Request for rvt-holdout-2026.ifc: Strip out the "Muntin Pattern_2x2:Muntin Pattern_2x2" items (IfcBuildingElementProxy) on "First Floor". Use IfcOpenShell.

First a look at what the model holds.

```python
import ifcopenshell
import ifcopenshell.util.element

model = ifcopenshell.open("rvt-holdout-2026.ifc")
print(model.schema)
storey = next(s for s in model.by_type("IfcBuildingStorey") if s.Name == "First Floor")
proxies = [e for e in ifcopenshell.util.element.get_decomposition(storey) if e.is_a("IfcBuildingElementProxy")]
seen = {}
for e in proxies:
    element_type = ifcopenshell.util.element.get_type(e)
    name = element_type.Name if element_type not in (None, e) else None
    seen[name] = seen.get(name, 0) + 1
for name, count in sorted(seen.items(), key=str):
    print(count, "x", name)
```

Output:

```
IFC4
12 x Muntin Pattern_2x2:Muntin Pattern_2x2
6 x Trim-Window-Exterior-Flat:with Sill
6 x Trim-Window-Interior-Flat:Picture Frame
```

```python
import ifcopenshell
import ifcopenshell.api.root
import ifcopenshell.util.element

model = ifcopenshell.open("rvt-holdout-2026.ifc")

storey = next(s for s in model.by_type("IfcBuildingStorey") if s.Name == "First Floor")
proxies = [e for e in ifcopenshell.util.element.get_decomposition(storey) if e.is_a("IfcBuildingElementProxy")]
targets = [e for e in proxies if (t := ifcopenshell.util.element.get_type(e)) not in (None, e) and t.Name == "Muntin Pattern_2x2:Muntin Pattern_2x2"]

for e in targets:
    ifcopenshell.api.root.remove_product(model, product=e)
print(len(targets), "removed")

model.write("rvt-holdout-2026_edited.ifc")
```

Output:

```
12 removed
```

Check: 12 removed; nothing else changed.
